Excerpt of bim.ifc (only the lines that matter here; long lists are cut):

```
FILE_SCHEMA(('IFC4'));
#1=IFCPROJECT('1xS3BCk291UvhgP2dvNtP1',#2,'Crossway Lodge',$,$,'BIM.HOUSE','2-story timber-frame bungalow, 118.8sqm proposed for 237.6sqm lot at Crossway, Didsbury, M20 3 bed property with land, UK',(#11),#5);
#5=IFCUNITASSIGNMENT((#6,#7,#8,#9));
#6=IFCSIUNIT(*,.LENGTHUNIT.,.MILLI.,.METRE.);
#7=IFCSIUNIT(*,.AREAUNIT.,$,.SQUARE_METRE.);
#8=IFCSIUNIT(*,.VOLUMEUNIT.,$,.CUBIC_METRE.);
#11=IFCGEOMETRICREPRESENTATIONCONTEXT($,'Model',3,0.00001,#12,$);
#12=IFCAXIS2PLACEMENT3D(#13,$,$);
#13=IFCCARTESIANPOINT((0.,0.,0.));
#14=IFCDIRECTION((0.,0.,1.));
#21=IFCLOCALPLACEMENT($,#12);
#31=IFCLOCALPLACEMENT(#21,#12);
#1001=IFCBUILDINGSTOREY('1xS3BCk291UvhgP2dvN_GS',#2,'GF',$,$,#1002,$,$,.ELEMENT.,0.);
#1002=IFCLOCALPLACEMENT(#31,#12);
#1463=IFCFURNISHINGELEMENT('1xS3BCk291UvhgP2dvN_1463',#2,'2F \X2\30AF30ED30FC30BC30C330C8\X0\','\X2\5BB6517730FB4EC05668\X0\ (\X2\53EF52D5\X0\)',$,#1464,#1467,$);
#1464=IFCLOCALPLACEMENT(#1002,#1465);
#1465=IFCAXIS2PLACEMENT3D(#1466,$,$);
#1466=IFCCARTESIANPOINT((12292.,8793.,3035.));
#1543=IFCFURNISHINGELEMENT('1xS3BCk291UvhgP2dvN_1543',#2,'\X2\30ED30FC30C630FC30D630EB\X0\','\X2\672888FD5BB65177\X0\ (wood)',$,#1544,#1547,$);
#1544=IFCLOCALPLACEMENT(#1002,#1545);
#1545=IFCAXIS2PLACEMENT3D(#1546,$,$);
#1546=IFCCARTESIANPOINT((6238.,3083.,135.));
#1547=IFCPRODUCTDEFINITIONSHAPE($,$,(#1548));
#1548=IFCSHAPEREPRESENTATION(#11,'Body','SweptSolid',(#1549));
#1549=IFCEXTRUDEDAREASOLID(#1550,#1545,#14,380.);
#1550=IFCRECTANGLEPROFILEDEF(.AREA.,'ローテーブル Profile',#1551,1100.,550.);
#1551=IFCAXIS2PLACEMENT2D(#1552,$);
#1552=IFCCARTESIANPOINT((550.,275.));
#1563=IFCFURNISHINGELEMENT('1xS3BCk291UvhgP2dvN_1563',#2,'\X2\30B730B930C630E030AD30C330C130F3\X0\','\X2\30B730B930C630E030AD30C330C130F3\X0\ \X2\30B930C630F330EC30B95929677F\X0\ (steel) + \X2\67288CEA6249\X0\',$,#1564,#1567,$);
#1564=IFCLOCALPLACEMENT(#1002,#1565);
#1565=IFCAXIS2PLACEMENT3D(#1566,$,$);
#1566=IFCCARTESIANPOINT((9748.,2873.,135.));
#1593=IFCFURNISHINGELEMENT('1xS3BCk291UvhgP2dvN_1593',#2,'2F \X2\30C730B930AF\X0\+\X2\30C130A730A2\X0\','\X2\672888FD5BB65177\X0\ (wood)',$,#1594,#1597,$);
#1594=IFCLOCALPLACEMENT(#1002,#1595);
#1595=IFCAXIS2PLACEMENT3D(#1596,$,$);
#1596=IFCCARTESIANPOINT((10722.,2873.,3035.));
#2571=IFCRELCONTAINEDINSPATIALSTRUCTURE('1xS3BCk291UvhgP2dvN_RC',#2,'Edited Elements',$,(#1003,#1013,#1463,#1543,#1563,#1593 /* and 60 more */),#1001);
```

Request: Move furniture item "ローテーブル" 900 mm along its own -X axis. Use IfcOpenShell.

```python
import ifcopenshell
import ifcopenshell.api.geometry
import ifcopenshell.util.placement

model = ifcopenshell.open("bim.ifc")

item = model.by_guid("1xS3BCk291UvhgP2dvN_1543")
matrix = ifcopenshell.util.placement.get_local_placement(item.ObjectPlacement)
matrix[:3, 3] -= matrix[:3, 0] * 900.0
ifcopenshell.api.geometry.edit_object_placement(model, product=item, matrix=matrix, is_si=False)

print(ifcopenshell.util.placement.get_local_placement(item.ObjectPlacement).round(3) + 0.0)

model.write("bim-out.ifc")
```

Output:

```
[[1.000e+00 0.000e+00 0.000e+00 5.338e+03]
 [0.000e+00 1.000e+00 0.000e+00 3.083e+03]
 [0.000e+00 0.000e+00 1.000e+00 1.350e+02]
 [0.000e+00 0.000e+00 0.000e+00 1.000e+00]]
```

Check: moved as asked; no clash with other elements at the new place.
